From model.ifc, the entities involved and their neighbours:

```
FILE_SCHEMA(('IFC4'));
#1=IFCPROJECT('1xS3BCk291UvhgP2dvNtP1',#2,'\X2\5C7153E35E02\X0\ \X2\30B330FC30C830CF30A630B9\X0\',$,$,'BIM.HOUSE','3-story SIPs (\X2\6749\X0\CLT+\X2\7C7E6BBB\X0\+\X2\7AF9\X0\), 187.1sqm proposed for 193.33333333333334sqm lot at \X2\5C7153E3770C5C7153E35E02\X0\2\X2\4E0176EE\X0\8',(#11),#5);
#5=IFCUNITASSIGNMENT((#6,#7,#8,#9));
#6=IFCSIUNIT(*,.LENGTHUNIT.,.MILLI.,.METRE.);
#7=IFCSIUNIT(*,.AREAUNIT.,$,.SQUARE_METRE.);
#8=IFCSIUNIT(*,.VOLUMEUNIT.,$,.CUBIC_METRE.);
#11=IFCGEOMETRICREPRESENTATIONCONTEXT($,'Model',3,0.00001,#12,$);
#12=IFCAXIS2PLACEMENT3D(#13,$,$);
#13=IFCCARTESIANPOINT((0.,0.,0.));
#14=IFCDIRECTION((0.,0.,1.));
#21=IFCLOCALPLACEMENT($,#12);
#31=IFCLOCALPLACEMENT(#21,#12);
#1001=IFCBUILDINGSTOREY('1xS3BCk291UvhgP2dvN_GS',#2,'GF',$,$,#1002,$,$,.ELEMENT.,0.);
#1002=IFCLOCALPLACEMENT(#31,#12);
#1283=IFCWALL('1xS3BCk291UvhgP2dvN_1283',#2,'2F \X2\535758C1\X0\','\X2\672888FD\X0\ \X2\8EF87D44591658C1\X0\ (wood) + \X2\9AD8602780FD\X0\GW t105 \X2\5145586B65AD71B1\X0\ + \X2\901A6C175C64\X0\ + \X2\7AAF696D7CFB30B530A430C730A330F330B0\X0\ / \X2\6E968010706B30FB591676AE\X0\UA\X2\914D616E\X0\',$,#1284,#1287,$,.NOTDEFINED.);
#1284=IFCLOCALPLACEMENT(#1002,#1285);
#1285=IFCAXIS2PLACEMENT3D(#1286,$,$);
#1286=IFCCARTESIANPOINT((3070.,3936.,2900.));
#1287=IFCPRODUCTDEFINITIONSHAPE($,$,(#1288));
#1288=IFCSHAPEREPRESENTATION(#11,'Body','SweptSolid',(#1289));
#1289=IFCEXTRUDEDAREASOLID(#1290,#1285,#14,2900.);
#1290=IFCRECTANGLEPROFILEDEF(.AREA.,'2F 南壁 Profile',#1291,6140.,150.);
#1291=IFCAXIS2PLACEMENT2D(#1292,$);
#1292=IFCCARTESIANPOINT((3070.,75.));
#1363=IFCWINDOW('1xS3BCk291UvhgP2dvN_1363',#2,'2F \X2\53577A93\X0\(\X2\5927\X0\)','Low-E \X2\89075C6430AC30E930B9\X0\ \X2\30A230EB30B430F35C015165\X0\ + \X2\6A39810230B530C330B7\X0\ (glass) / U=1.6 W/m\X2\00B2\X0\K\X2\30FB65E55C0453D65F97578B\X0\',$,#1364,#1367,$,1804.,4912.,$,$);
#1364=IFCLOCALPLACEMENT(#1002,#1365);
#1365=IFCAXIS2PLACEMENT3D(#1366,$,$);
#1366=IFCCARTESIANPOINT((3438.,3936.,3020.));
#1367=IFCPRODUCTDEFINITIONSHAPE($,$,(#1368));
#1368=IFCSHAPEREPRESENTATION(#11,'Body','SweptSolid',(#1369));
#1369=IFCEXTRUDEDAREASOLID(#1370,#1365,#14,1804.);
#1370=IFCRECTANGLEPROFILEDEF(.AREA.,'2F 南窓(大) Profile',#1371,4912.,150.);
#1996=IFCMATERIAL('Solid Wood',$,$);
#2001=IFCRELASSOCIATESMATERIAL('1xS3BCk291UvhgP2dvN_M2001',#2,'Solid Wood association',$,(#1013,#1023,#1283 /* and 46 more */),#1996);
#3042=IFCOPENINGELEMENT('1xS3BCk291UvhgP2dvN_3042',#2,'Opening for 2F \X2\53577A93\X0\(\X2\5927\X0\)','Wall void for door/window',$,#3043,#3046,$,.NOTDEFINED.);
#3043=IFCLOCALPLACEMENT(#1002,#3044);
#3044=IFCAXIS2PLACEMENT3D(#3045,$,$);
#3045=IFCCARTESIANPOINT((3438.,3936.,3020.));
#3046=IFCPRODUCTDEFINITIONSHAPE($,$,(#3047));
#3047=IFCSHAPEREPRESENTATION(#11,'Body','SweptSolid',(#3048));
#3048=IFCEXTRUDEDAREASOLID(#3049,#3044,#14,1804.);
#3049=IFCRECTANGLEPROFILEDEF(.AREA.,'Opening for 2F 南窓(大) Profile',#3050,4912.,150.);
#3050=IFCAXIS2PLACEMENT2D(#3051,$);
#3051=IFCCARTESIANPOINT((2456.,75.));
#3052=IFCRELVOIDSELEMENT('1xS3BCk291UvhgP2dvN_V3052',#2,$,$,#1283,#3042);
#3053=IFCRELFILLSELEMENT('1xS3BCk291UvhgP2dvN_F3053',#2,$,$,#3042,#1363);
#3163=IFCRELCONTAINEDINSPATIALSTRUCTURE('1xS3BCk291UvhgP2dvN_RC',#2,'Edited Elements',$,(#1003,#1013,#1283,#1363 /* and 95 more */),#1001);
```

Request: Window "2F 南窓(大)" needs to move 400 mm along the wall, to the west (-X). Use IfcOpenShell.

```python
import ifcopenshell
import ifcopenshell.api.geometry
import ifcopenshell.util.placement
import ifcopenshell.util.unit

model = ifcopenshell.open("model.ifc")
unit_scale = ifcopenshell.util.unit.calculate_unit_scale(model)

window = model.by_guid("1xS3BCk291UvhgP2dvN_1363")
opening = window.FillsVoids[0].RelatingOpeningElement
wall = opening.VoidsElements[0].RelatingBuildingElement

wall_matrix = ifcopenshell.util.placement.get_local_placement(wall.ObjectPlacement)
shift = wall_matrix[:3, 0] * -0.4 / unit_scale
before = ifcopenshell.util.placement.get_local_placement(window.ObjectPlacement)[:3, 3].copy()

# The window is not placed relative to its opening, so move both.
for product in (opening, window):
    matrix = ifcopenshell.util.placement.get_local_placement(product.ObjectPlacement)
    matrix[:3, 3] += shift
    ifcopenshell.api.geometry.edit_object_placement(model, product=product, matrix=matrix, is_si=False)

after = ifcopenshell.util.placement.get_local_placement(window.ObjectPlacement)[:3, 3]
print("window moved by", (after - before).round(3) + 0.0)

model.write("model_edited.ifc")
```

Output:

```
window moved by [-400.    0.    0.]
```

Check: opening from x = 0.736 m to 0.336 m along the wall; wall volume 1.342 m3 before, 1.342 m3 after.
